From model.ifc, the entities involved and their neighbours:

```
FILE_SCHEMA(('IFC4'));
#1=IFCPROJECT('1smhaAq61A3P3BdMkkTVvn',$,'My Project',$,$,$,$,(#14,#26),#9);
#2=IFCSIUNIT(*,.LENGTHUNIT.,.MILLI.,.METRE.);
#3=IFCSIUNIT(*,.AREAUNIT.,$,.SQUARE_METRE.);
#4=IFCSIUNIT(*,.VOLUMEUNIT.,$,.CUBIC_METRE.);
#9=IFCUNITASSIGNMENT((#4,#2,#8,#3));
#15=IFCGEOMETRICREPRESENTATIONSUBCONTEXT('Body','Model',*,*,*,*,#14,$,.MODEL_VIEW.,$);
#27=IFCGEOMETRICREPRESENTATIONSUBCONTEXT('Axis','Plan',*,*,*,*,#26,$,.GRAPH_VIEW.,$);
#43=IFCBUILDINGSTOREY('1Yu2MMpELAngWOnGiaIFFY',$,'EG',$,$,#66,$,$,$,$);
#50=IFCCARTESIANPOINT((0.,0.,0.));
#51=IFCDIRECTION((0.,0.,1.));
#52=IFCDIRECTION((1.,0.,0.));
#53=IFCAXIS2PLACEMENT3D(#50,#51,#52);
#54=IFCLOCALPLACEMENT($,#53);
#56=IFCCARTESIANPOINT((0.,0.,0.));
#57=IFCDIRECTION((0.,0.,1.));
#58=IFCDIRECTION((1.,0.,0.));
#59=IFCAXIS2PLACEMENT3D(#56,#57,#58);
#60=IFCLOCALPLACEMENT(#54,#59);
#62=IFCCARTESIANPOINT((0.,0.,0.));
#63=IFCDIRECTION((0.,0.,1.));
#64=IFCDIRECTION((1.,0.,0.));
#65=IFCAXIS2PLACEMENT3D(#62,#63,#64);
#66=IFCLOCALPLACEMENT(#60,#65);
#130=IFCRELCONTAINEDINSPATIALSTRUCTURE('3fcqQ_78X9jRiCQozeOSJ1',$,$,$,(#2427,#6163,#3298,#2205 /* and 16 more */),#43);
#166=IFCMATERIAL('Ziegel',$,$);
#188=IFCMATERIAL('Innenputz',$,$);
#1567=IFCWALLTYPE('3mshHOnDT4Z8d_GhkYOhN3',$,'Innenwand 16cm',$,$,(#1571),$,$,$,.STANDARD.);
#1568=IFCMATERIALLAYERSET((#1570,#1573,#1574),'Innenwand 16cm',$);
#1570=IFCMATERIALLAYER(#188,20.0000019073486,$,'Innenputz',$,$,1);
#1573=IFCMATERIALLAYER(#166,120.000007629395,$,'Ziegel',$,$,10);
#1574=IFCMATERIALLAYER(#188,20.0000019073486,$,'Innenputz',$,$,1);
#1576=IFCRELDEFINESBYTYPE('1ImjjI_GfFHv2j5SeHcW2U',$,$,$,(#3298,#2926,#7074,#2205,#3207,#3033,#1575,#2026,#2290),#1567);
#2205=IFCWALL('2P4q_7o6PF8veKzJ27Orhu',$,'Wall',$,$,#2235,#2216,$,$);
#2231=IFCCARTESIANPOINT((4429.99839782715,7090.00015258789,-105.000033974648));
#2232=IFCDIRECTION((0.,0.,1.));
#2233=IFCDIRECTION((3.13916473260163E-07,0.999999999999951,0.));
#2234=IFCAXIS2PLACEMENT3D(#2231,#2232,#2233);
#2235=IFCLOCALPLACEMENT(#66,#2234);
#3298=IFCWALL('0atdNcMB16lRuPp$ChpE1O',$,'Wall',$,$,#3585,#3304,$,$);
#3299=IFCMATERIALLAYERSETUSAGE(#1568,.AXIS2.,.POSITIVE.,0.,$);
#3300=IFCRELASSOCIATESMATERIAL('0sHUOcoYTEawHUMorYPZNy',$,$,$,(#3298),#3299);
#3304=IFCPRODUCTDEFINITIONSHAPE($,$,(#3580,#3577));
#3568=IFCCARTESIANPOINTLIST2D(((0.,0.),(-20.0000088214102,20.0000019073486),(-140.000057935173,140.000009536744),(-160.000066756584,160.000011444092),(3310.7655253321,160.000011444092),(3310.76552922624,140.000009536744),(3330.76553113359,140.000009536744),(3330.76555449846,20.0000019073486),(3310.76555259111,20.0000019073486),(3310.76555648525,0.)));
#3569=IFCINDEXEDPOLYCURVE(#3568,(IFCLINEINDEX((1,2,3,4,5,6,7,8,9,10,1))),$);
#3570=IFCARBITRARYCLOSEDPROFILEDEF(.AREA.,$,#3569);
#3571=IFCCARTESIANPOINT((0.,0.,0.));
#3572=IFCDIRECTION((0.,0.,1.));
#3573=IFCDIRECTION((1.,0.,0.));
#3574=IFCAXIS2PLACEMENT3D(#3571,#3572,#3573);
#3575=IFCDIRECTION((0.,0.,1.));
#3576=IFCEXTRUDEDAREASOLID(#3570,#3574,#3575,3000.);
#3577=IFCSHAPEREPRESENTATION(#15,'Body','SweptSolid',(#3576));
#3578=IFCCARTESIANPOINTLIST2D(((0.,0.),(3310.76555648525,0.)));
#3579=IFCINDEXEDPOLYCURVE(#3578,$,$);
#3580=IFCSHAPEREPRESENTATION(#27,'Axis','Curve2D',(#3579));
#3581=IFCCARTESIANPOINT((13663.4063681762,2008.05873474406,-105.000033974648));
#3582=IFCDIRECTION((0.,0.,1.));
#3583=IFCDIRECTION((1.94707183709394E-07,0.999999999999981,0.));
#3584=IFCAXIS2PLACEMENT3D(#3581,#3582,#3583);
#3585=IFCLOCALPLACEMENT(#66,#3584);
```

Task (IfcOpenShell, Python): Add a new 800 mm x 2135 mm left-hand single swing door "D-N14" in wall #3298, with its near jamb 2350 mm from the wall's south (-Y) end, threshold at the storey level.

```python
import numpy as np
import ifcopenshell
import ifcopenshell.api.feature
import ifcopenshell.api.geometry
import ifcopenshell.api.root
import ifcopenshell.api.spatial
import ifcopenshell.geom
import ifcopenshell.util.element
import ifcopenshell.util.placement
import ifcopenshell.util.representation
import ifcopenshell.util.shape
import ifcopenshell.util.unit

model = ifcopenshell.open("model.ifc")
unit_scale = ifcopenshell.util.unit.calculate_unit_scale(model)
settings = ifcopenshell.geom.settings()


def volume(element):
    """Net volume in cubic metres, openings subtracted."""
    shape = ifcopenshell.geom.create_shape(settings, element)
    return ifcopenshell.util.shape.get_volume(shape.geometry)


wall = model.by_guid("0atdNcMB16lRuPp$ChpE1O")
storey = ifcopenshell.util.element.get_container(wall, ifc_class="IfcBuildingStorey")
context = ifcopenshell.util.representation.get_context(model, "Model", "Body", "MODEL_VIEW")
before = volume(wall)

width, height, from_end, sill = 0.8, 2.135, 2.35, 0.0  # metres

# The wall runs along its own X axis, and the end named is its -X end.
wall_shape = ifcopenshell.geom.create_shape(settings, wall)
x, y, z = ifcopenshell.util.shape.get_vertices(wall_shape.geometry).T
start = x.min() + from_end
face, thickness = float(y.min()), float(y.max() - y.min())
wall_matrix = ifcopenshell.util.placement.get_local_placement(wall.ObjectPlacement)
level = ifcopenshell.util.placement.get_local_placement(storey.ObjectPlacement)[2, 3]


def in_wall(x, y):
    """Placement at x, y metres in the wall's axes, at sill height."""
    matrix = wall_matrix.copy()
    matrix[:, 3] = wall_matrix @ np.array([x / unit_scale, y / unit_scale, 0.0, 1.0])
    matrix[2, 3] = level + sill / unit_scale
    return matrix


# Opening: a box that overshoots both wall faces by 50 mm.
opening = ifcopenshell.api.root.create_entity(model, ifc_class="IfcOpeningElement", predefined_type="OPENING")
box = ifcopenshell.api.geometry.add_wall_representation(
    model, context=context, length=width, height=height, thickness=thickness + 0.1
)
ifcopenshell.api.geometry.assign_representation(model, product=opening, representation=box)
ifcopenshell.api.geometry.edit_object_placement(model, product=opening, matrix=in_wall(start, face - 0.05), is_si=False)
ifcopenshell.api.feature.add_feature(model, feature=opening, element=wall)

door = ifcopenshell.api.root.create_entity(model, ifc_class="IfcDoor", name="D-N14", predefined_type="DOOR")
door.OverallWidth, door.OverallHeight = width / unit_scale, height / unit_scale
door.OperationType = "SINGLE_SWING_LEFT"
body = ifcopenshell.api.geometry.add_door_representation(
    model,
    context=context,
    overall_width=door.OverallWidth,
    overall_height=door.OverallHeight,
    operation_type="SINGLE_SWING_LEFT",
    lining_properties={"LiningDepth": thickness / unit_scale, "ThresholdDepth": thickness / unit_scale},
)
ifcopenshell.api.geometry.assign_representation(model, product=door, representation=body)
ifcopenshell.api.spatial.assign_container(model, products=[door], relating_structure=storey)
ifcopenshell.api.feature.add_filling(model, opening=opening, element=door)

# The lining spans the wall, so the door starts at the wall face.
ifcopenshell.api.geometry.edit_object_placement(model, product=door, matrix=in_wall(start, face), is_si=False)

after = volume(wall)

print(f"wall volume {before:.3f} -> {after:.3f} m3")

model.write("model_updated.ifc")
```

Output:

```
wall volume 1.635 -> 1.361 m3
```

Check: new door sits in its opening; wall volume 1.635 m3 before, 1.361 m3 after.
